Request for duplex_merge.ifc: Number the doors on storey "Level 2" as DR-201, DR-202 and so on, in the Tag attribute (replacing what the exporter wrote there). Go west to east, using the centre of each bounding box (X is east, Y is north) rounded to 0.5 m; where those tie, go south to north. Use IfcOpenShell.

First a look at what the model holds.

```python
import ifcopenshell
import ifcopenshell.util.element
import ifcopenshell.util.placement

model = ifcopenshell.open("duplex_merge.ifc")
print(model.schema)
storey = next(s for s in model.by_type("IfcBuildingStorey") if s.Name == "Level 2")
doors = [e for e in ifcopenshell.util.element.get_decomposition(storey) if e.is_a("IfcDoor")]
for e in sorted(doors, key=lambda e: e.id()):
    origin = ifcopenshell.util.placement.get_local_placement(e.ObjectPlacement)[:3, 3]
    print(e.id(), e.Tag, e.Name, origin.round(2) + 0.0, sep=" | ")
```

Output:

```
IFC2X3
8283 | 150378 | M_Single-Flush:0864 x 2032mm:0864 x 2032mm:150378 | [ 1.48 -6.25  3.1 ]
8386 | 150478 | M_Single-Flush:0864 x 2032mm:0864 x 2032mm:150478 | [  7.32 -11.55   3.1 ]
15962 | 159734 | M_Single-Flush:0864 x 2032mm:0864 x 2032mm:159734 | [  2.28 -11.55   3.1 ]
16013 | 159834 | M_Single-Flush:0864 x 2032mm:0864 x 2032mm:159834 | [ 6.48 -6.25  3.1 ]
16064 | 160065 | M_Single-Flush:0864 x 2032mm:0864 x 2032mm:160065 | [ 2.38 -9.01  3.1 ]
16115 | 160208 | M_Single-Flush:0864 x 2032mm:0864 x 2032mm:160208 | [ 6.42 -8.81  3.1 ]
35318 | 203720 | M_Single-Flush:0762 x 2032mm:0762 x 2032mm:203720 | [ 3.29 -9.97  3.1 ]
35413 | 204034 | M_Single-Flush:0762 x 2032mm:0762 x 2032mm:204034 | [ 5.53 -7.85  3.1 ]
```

```python
import ifcopenshell
import ifcopenshell.geom
import ifcopenshell.util.element
import ifcopenshell.util.shape

model = ifcopenshell.open("duplex_merge.ifc")
settings = ifcopenshell.geom.settings()
settings.set("use-world-coords", True)


def centre(element):
    shape = ifcopenshell.geom.create_shape(settings, element)
    return ifcopenshell.util.shape.get_bbox_centroid(shape.geometry)


storey = next(s for s in model.by_type("IfcBuildingStorey") if s.Name == "Level 2")
doors = [e for e in ifcopenshell.util.element.get_decomposition(storey) if e.is_a("IfcDoor")]

# Insertion points can sit at a corner or the storey origin, so sort by the geometry (in metres).
centres = {e: centre(e) for e in doors}
doors.sort(key=lambda e: (round(centres[e][0] / 0.5), centres[e][1]))

for i, e in enumerate(doors, start=1):
    number = f"DR-2{i:02d}"
    e.Tag = number
    print(e.id(), number)

model.write("duplex_merge_rev.ifc")
```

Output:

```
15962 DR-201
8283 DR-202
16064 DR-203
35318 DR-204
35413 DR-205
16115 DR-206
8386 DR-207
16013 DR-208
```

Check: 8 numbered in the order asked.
